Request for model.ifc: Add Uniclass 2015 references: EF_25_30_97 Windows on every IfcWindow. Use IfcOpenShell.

First a look at what the model holds.

```python
import ifcopenshell

model = ifcopenshell.open("model.ifc")
print(model.schema)
print("classifications:", [c.Name for c in model.by_type("IfcClassification")])
for ifc_class in ("IfcDoor", "IfcRoof", "IfcStair", "IfcWall", "IfcWindow"):
    print(ifc_class, len(model.by_type(ifc_class)))
```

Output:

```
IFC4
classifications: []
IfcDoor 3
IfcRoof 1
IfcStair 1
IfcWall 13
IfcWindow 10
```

```python
import ifcopenshell
import ifcopenshell.api.classification

model = ifcopenshell.open("model.ifc")

system = ifcopenshell.api.classification.add_classification(model, classification="Uniclass 2015")

codes = {
    "IfcWindow": ("EF_25_30_97", "Windows"),
}
for ifc_class, (code, name) in codes.items():
    products = model.by_type(ifc_class)
    ifcopenshell.api.classification.add_reference(
        model, products=products, classification=system, identification=code, name=name
    )
    print(code, len(products))

model.write("model_edited.ifc")
```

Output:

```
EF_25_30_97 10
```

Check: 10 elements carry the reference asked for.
